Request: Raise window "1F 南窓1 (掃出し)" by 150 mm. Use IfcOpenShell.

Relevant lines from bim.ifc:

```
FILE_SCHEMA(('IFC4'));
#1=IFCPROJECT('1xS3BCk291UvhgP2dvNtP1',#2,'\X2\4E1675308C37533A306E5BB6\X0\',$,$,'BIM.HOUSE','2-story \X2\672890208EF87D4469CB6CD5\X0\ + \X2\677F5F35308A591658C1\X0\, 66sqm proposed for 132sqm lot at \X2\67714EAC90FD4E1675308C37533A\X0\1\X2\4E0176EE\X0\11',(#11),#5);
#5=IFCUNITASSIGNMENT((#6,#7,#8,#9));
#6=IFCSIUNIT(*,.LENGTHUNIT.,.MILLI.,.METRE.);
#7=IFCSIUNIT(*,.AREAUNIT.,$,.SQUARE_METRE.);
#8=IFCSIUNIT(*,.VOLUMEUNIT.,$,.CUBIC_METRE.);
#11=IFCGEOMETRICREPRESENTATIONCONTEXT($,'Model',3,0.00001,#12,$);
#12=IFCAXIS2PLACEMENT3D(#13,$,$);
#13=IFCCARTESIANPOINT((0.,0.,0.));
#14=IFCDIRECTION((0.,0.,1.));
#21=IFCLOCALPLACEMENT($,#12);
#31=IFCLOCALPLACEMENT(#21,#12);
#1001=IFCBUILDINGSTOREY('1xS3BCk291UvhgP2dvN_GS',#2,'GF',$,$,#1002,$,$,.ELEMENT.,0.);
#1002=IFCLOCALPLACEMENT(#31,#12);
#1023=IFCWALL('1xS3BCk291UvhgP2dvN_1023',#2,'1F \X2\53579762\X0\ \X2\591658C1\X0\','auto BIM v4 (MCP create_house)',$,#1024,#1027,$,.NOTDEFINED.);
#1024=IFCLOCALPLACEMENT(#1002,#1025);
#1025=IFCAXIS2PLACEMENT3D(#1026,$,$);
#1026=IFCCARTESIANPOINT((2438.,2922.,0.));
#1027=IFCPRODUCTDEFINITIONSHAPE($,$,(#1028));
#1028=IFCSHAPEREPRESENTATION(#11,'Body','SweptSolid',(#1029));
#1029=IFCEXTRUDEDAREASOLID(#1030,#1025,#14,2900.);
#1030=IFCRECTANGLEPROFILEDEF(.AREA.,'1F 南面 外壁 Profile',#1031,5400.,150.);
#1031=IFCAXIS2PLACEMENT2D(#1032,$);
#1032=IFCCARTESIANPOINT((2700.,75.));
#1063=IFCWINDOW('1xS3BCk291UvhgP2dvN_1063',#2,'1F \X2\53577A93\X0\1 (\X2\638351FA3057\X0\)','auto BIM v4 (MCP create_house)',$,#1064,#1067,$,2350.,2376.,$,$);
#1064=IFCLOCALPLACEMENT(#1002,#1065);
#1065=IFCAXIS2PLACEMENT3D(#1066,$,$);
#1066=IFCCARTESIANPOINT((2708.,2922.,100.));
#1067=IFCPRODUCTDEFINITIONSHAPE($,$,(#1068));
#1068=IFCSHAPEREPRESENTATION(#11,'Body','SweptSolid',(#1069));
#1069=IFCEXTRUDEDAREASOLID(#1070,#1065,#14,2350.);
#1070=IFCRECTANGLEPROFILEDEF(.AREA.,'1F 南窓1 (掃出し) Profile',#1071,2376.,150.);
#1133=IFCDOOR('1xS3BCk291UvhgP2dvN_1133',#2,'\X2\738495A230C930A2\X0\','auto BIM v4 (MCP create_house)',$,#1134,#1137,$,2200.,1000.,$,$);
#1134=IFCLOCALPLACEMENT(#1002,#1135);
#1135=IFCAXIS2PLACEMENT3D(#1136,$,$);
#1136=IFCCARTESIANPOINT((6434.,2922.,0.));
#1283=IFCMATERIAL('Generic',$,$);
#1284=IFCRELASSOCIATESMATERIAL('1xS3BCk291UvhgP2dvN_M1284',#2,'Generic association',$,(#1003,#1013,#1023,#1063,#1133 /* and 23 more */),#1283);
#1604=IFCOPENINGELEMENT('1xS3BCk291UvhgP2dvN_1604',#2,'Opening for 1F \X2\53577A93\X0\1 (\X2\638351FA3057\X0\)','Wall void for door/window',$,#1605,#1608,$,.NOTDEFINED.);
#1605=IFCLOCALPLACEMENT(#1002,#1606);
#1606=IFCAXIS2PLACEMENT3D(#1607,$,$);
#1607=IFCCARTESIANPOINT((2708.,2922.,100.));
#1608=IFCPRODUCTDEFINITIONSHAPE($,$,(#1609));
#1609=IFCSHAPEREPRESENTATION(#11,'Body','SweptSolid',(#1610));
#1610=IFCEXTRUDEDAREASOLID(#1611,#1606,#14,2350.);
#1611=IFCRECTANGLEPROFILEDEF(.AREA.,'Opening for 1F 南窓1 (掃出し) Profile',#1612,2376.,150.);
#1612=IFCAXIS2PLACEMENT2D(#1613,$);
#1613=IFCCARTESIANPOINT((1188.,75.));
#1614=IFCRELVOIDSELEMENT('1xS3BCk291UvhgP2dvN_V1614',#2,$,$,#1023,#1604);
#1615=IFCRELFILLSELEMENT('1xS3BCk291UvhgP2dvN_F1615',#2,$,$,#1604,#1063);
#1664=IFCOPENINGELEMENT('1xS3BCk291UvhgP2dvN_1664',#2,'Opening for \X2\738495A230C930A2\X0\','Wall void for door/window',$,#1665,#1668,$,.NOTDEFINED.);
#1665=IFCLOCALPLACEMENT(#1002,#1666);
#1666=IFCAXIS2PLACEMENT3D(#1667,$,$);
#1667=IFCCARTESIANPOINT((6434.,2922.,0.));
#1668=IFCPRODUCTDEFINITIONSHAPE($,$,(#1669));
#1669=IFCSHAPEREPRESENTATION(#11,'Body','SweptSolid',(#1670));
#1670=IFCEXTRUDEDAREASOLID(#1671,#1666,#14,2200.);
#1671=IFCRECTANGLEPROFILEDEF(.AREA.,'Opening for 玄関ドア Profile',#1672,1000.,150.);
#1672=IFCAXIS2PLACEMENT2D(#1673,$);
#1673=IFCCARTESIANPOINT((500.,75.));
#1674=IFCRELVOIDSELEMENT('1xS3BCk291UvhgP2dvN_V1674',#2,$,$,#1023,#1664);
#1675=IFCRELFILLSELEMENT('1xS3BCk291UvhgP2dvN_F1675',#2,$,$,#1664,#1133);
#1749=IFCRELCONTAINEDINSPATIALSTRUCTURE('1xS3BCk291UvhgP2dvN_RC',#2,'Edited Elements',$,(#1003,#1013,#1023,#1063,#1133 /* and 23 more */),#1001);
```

```python
import numpy as np
import ifcopenshell
import ifcopenshell.api.geometry
import ifcopenshell.util.placement
import ifcopenshell.util.unit

model = ifcopenshell.open("bim.ifc")
unit_scale = ifcopenshell.util.unit.calculate_unit_scale(model)

window = model.by_guid("1xS3BCk291UvhgP2dvN_1063")
opening = window.FillsVoids[0].RelatingOpeningElement
dz = 150.0

shift = np.array([0.0, 0.0, dz])
# The window is not placed relative to its opening, so move both.
for product in (opening, window):
    matrix = ifcopenshell.util.placement.get_local_placement(product.ObjectPlacement)
    matrix[:3, 3] += shift
    ifcopenshell.api.geometry.edit_object_placement(model, product=product, matrix=matrix, is_si=False)

print(f"moved by {dz * unit_scale:+.3f} m")

model.write("bim_edited.ifc")
```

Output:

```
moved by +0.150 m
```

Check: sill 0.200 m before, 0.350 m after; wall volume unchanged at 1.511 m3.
